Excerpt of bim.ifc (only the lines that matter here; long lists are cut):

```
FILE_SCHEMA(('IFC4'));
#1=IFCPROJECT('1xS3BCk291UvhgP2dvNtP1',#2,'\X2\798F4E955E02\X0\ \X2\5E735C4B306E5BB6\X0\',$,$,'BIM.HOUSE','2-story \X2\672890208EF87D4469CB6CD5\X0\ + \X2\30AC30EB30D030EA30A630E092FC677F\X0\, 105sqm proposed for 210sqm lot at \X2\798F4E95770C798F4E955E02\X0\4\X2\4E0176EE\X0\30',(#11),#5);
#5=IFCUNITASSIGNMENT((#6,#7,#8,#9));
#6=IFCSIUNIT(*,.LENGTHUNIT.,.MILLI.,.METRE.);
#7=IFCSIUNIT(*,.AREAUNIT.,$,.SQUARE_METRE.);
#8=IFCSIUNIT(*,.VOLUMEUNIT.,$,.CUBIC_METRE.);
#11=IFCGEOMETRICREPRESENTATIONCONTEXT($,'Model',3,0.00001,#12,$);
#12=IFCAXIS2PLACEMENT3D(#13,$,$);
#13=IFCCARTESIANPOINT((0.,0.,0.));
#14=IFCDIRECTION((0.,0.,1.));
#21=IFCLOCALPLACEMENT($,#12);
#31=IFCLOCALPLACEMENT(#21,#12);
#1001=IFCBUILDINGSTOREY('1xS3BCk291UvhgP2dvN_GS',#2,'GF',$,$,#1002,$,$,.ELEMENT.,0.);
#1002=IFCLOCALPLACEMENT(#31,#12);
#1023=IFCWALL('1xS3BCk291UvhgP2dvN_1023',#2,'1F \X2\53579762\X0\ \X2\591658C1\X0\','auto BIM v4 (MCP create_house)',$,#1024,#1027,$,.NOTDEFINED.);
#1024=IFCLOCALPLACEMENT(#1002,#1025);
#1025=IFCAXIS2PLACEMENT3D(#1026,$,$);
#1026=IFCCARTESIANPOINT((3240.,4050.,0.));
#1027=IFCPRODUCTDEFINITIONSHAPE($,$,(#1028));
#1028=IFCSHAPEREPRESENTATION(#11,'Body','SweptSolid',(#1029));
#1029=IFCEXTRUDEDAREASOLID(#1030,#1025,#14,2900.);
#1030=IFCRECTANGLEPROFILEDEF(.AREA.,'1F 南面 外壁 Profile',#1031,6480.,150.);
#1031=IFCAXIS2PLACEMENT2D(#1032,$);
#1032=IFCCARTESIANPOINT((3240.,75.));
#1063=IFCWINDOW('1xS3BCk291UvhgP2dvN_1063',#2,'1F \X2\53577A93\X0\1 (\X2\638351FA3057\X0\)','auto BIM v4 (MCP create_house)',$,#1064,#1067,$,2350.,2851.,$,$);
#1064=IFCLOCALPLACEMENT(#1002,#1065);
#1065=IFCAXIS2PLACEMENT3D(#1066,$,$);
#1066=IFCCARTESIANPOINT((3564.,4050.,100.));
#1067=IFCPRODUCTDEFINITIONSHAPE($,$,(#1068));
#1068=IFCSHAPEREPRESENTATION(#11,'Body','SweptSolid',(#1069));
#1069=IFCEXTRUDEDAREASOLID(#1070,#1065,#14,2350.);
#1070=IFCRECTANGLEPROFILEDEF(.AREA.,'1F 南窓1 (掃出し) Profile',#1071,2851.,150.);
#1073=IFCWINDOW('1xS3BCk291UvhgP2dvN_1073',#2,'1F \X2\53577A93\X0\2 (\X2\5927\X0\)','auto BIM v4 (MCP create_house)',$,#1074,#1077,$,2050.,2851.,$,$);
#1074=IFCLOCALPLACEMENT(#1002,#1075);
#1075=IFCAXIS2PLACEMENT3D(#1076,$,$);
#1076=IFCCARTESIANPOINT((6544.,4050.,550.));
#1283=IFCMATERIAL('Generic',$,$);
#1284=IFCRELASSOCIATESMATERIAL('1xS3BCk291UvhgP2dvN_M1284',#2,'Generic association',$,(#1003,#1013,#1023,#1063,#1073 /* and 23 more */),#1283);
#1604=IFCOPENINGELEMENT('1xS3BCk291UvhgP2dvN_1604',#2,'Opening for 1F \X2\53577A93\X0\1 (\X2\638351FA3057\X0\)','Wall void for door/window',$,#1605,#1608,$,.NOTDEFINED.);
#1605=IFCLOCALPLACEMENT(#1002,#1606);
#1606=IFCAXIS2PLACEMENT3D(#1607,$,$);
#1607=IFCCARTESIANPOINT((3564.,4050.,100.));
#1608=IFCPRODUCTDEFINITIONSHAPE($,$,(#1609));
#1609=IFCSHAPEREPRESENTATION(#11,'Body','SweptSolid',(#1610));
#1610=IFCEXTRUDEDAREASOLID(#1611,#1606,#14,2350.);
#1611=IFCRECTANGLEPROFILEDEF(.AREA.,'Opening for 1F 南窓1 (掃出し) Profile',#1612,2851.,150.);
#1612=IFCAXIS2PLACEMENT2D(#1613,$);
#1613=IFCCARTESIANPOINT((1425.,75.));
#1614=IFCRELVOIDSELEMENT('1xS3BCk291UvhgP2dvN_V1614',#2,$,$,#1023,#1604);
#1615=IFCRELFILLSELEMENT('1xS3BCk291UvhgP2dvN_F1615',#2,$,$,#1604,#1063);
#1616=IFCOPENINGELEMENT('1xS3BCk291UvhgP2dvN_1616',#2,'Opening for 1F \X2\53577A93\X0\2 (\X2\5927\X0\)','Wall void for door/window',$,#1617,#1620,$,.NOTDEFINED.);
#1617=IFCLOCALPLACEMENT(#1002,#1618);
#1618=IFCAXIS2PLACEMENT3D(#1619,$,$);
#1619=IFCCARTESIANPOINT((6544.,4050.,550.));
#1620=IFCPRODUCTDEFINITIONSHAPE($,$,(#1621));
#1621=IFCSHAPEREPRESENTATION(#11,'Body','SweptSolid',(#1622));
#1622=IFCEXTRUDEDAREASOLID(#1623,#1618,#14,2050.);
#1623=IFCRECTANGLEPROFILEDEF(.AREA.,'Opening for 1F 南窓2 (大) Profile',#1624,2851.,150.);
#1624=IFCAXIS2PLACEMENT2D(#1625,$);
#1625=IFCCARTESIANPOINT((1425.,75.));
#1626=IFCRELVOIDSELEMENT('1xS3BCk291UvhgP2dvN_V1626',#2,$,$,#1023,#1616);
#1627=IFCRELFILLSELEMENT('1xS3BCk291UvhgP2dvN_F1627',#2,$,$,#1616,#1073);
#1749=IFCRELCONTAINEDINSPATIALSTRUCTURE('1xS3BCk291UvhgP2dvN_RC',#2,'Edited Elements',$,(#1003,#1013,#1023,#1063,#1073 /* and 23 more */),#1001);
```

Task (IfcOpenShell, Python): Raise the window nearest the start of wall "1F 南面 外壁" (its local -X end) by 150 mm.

```python
import numpy as np
import ifcopenshell
import ifcopenshell.api.geometry
import ifcopenshell.util.placement
import ifcopenshell.util.unit

model = ifcopenshell.open("bim.ifc")
unit_scale = ifcopenshell.util.unit.calculate_unit_scale(model)

window = model.by_guid("1xS3BCk291UvhgP2dvN_1063")
opening = window.FillsVoids[0].RelatingOpeningElement
dz = 150.0

shift = np.array([0.0, 0.0, dz])
# The window is not placed relative to its opening, so move both.
for product in (opening, window):
    matrix = ifcopenshell.util.placement.get_local_placement(product.ObjectPlacement)
    matrix[:3, 3] += shift
    ifcopenshell.api.geometry.edit_object_placement(model, product=product, matrix=matrix, is_si=False)

print(f"moved by {dz * unit_scale:+.3f} m")

model.write("bim-out.ifc")
```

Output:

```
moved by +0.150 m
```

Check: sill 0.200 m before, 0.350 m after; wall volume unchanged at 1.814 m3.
